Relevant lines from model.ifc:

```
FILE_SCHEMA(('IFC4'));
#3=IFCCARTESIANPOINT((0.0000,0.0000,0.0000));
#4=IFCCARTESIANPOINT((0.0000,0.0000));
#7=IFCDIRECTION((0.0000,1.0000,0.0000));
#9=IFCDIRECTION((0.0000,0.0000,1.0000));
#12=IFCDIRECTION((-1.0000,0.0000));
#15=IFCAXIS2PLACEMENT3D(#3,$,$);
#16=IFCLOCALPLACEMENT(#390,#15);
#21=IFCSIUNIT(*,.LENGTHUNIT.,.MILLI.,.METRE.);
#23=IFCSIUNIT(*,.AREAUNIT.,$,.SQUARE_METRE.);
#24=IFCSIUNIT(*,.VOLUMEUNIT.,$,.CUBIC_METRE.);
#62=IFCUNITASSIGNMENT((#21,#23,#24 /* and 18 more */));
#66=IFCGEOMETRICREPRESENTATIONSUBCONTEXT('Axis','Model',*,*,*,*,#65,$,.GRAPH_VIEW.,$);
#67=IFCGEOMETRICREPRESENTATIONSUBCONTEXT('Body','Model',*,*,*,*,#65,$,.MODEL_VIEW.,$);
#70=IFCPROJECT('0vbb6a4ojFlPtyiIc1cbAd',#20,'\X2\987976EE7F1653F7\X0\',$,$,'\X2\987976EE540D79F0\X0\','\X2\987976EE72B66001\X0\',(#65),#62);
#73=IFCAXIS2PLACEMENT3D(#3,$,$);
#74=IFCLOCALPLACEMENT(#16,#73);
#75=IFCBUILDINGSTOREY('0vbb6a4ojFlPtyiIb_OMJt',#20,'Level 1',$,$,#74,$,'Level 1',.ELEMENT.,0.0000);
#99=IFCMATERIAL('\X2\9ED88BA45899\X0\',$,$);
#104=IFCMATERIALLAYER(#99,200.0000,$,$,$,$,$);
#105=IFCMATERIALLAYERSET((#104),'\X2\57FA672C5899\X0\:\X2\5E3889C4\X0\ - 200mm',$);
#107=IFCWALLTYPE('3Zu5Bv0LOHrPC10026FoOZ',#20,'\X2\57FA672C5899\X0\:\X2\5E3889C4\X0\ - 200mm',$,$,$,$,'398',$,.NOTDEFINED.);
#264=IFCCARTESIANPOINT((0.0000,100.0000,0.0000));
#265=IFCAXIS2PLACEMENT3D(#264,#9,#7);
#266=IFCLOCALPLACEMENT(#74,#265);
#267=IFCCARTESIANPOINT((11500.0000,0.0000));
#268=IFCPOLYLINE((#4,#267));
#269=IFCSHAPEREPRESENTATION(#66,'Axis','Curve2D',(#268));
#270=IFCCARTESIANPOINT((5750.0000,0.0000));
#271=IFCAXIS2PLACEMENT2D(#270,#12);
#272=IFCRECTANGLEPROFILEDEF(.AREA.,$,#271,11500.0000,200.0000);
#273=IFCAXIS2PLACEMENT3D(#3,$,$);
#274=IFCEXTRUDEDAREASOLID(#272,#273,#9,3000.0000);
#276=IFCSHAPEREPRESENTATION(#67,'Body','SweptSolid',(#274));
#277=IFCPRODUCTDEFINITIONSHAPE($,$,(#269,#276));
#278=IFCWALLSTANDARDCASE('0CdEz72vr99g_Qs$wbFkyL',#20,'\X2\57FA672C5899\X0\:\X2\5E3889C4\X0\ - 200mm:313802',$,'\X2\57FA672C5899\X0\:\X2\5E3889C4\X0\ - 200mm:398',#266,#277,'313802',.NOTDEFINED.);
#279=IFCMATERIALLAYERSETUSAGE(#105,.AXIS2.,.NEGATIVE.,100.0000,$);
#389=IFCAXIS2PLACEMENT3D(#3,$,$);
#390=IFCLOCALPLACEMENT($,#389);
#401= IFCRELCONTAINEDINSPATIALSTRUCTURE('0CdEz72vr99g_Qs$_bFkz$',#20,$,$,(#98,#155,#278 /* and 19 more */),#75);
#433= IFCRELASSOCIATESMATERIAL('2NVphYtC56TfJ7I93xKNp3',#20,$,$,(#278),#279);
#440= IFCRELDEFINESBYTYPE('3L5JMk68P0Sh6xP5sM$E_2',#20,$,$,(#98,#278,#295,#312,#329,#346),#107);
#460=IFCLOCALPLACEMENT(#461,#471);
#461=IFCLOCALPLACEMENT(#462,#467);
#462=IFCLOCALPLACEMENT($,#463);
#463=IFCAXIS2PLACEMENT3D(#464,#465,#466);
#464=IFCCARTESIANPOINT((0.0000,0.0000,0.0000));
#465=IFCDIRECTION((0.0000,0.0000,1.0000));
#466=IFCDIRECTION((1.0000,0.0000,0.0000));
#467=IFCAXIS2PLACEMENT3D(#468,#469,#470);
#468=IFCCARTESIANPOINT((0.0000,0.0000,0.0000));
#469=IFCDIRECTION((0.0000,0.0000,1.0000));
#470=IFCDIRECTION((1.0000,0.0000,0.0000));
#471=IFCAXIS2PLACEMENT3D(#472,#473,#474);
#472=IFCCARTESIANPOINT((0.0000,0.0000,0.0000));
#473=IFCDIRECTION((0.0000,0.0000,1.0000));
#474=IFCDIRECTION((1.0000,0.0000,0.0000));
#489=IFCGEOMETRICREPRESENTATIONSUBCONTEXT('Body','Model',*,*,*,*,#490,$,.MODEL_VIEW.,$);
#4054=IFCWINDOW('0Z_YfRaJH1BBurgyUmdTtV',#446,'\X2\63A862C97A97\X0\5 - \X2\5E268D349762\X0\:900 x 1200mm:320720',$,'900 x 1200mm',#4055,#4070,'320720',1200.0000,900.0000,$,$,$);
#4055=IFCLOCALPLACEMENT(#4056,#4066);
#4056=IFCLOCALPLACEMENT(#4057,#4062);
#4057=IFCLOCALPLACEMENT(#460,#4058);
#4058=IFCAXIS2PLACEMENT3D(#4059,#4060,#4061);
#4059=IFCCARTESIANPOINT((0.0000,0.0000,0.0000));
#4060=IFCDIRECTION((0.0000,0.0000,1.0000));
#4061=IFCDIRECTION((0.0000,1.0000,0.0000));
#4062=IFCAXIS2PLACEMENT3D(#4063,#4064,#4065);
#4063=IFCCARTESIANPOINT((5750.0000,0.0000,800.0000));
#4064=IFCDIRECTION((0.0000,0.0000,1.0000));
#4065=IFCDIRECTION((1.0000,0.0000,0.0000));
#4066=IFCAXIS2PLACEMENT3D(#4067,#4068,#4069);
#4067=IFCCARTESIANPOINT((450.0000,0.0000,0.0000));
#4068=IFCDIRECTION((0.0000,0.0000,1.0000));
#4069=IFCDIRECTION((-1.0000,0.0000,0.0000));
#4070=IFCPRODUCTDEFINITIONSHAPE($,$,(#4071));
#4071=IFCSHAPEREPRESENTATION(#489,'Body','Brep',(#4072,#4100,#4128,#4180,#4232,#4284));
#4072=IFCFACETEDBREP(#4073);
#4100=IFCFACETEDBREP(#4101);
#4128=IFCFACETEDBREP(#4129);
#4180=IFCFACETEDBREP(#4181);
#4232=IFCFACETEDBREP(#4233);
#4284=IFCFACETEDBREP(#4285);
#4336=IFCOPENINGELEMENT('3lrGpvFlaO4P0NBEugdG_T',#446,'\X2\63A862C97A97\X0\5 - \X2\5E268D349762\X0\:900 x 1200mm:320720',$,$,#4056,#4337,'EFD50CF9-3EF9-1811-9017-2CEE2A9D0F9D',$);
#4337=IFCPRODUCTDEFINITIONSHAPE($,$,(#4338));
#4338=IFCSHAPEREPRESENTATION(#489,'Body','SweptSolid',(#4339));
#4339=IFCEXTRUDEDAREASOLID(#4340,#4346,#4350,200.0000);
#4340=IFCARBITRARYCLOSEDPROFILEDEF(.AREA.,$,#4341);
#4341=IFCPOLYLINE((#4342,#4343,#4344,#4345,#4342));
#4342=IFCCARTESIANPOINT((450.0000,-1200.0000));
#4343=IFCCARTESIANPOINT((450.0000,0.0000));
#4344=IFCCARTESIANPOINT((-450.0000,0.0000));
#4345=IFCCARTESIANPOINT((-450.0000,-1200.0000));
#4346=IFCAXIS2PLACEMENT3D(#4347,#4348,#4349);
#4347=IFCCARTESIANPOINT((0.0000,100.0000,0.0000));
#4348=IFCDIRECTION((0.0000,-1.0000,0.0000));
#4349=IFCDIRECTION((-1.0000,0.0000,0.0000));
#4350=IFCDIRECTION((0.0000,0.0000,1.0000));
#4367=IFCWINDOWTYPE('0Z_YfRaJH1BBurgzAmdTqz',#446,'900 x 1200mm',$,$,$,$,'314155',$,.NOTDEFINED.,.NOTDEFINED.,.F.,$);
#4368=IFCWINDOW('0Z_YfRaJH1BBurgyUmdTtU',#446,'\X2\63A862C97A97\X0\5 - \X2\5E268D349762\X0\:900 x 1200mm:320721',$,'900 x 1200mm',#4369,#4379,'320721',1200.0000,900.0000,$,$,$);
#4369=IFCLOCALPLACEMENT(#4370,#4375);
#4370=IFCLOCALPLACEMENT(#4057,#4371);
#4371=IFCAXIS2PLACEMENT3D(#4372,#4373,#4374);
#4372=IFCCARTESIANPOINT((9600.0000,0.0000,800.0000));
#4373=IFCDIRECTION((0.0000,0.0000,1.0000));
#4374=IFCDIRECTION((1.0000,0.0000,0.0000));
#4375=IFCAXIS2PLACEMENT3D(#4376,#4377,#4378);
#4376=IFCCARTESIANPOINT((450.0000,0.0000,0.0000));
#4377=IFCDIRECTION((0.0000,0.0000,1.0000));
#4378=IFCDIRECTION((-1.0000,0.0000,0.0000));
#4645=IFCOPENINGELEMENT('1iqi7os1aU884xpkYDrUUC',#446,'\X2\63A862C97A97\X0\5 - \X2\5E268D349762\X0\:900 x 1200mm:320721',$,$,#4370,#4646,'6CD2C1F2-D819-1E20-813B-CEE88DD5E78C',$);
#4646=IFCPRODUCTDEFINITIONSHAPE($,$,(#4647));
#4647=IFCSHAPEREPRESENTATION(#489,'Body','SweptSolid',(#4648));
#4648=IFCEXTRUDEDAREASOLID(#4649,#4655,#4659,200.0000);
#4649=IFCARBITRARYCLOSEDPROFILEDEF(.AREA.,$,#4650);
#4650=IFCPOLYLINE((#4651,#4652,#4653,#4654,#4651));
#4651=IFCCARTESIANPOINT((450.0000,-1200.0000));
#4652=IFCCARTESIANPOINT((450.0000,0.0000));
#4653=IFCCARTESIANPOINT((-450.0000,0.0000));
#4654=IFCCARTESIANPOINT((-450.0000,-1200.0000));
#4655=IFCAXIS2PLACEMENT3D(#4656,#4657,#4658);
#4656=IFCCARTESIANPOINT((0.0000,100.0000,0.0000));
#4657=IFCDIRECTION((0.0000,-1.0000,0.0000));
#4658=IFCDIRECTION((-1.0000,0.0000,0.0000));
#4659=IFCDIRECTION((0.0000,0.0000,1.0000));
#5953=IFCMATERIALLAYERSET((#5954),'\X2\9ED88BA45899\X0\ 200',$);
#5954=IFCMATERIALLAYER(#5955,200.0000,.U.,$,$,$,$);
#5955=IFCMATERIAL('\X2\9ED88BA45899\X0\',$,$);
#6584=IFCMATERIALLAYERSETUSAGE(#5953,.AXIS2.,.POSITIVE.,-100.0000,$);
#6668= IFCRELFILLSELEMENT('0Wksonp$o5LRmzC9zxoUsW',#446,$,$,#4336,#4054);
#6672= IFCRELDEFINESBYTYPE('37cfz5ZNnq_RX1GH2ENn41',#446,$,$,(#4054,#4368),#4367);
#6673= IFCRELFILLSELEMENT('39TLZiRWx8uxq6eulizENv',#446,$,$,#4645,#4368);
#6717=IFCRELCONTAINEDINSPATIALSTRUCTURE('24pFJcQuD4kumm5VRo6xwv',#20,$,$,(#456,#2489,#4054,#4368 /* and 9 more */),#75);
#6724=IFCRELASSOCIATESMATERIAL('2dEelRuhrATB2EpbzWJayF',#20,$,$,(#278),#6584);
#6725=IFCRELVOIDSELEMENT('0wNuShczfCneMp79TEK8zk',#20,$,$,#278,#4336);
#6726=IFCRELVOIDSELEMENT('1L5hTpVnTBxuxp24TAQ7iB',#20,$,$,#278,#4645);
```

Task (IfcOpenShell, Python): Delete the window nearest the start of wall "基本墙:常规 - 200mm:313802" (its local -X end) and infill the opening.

```python
import ifcopenshell
import ifcopenshell.api.feature
import ifcopenshell.api.root
import ifcopenshell.geom
import ifcopenshell.util.shape

model = ifcopenshell.open("model.ifc")
settings = ifcopenshell.geom.settings()


def volume(element):
    """Net volume in cubic metres, openings subtracted."""
    shape = ifcopenshell.geom.create_shape(settings, element)
    return ifcopenshell.util.shape.get_volume(shape.geometry)


window = model.by_id(4054)
opening = window.FillsVoids[0].RelatingOpeningElement
wall = opening.VoidsElements[0].RelatingBuildingElement
before = volume(wall)

ifcopenshell.api.root.remove_product(model, product=window)
ifcopenshell.api.feature.remove_feature(model, feature=opening)

after = volume(wall)

print(f"wall volume {before:.3f} -> {after:.3f} m3")

model.write("model_updated.ifc")
```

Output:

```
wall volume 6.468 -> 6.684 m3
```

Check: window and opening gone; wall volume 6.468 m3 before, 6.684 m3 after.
